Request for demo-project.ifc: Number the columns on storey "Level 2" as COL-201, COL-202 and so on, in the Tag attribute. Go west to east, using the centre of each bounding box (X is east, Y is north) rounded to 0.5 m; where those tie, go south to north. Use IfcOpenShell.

First a look at what the model holds.

```python
import ifcopenshell
import ifcopenshell.util.element
import ifcopenshell.util.placement

model = ifcopenshell.open("demo-project.ifc")
print(model.schema)
storey = next(s for s in model.by_type("IfcBuildingStorey") if s.Name == "Level 2")
columns = [e for e in ifcopenshell.util.element.get_decomposition(storey) if e.is_a("IfcColumn")]
for e in sorted(columns, key=lambda e: e.id()):
    origin = ifcopenshell.util.placement.get_local_placement(e.ObjectPlacement)[:3, 3]
    print(e.id(), e.Tag, e.Name, origin.round(2) + 0.0, sep=" | ")
```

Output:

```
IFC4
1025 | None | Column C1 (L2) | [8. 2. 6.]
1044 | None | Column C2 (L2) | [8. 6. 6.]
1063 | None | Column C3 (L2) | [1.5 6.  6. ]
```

```python
import ifcopenshell
import ifcopenshell.geom
import ifcopenshell.util.element
import ifcopenshell.util.shape

model = ifcopenshell.open("demo-project.ifc")
settings = ifcopenshell.geom.settings()
settings.set("use-world-coords", True)


def centre(element):
    shape = ifcopenshell.geom.create_shape(settings, element)
    return ifcopenshell.util.shape.get_bbox_centroid(shape.geometry)


storey = next(s for s in model.by_type("IfcBuildingStorey") if s.Name == "Level 2")
columns = [e for e in ifcopenshell.util.element.get_decomposition(storey) if e.is_a("IfcColumn")]

# Insertion points can sit at a corner or the storey origin, so sort by the geometry (in metres).
centres = {e: centre(e) for e in columns}
columns.sort(key=lambda e: (round(centres[e][0] / 0.5), centres[e][1]))

for i, e in enumerate(columns, start=1):
    number = f"COL-2{i:02d}"
    e.Tag = number
    print(e.id(), number)

model.write("demo-project_edited.ifc")
```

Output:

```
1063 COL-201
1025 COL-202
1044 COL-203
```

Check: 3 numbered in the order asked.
